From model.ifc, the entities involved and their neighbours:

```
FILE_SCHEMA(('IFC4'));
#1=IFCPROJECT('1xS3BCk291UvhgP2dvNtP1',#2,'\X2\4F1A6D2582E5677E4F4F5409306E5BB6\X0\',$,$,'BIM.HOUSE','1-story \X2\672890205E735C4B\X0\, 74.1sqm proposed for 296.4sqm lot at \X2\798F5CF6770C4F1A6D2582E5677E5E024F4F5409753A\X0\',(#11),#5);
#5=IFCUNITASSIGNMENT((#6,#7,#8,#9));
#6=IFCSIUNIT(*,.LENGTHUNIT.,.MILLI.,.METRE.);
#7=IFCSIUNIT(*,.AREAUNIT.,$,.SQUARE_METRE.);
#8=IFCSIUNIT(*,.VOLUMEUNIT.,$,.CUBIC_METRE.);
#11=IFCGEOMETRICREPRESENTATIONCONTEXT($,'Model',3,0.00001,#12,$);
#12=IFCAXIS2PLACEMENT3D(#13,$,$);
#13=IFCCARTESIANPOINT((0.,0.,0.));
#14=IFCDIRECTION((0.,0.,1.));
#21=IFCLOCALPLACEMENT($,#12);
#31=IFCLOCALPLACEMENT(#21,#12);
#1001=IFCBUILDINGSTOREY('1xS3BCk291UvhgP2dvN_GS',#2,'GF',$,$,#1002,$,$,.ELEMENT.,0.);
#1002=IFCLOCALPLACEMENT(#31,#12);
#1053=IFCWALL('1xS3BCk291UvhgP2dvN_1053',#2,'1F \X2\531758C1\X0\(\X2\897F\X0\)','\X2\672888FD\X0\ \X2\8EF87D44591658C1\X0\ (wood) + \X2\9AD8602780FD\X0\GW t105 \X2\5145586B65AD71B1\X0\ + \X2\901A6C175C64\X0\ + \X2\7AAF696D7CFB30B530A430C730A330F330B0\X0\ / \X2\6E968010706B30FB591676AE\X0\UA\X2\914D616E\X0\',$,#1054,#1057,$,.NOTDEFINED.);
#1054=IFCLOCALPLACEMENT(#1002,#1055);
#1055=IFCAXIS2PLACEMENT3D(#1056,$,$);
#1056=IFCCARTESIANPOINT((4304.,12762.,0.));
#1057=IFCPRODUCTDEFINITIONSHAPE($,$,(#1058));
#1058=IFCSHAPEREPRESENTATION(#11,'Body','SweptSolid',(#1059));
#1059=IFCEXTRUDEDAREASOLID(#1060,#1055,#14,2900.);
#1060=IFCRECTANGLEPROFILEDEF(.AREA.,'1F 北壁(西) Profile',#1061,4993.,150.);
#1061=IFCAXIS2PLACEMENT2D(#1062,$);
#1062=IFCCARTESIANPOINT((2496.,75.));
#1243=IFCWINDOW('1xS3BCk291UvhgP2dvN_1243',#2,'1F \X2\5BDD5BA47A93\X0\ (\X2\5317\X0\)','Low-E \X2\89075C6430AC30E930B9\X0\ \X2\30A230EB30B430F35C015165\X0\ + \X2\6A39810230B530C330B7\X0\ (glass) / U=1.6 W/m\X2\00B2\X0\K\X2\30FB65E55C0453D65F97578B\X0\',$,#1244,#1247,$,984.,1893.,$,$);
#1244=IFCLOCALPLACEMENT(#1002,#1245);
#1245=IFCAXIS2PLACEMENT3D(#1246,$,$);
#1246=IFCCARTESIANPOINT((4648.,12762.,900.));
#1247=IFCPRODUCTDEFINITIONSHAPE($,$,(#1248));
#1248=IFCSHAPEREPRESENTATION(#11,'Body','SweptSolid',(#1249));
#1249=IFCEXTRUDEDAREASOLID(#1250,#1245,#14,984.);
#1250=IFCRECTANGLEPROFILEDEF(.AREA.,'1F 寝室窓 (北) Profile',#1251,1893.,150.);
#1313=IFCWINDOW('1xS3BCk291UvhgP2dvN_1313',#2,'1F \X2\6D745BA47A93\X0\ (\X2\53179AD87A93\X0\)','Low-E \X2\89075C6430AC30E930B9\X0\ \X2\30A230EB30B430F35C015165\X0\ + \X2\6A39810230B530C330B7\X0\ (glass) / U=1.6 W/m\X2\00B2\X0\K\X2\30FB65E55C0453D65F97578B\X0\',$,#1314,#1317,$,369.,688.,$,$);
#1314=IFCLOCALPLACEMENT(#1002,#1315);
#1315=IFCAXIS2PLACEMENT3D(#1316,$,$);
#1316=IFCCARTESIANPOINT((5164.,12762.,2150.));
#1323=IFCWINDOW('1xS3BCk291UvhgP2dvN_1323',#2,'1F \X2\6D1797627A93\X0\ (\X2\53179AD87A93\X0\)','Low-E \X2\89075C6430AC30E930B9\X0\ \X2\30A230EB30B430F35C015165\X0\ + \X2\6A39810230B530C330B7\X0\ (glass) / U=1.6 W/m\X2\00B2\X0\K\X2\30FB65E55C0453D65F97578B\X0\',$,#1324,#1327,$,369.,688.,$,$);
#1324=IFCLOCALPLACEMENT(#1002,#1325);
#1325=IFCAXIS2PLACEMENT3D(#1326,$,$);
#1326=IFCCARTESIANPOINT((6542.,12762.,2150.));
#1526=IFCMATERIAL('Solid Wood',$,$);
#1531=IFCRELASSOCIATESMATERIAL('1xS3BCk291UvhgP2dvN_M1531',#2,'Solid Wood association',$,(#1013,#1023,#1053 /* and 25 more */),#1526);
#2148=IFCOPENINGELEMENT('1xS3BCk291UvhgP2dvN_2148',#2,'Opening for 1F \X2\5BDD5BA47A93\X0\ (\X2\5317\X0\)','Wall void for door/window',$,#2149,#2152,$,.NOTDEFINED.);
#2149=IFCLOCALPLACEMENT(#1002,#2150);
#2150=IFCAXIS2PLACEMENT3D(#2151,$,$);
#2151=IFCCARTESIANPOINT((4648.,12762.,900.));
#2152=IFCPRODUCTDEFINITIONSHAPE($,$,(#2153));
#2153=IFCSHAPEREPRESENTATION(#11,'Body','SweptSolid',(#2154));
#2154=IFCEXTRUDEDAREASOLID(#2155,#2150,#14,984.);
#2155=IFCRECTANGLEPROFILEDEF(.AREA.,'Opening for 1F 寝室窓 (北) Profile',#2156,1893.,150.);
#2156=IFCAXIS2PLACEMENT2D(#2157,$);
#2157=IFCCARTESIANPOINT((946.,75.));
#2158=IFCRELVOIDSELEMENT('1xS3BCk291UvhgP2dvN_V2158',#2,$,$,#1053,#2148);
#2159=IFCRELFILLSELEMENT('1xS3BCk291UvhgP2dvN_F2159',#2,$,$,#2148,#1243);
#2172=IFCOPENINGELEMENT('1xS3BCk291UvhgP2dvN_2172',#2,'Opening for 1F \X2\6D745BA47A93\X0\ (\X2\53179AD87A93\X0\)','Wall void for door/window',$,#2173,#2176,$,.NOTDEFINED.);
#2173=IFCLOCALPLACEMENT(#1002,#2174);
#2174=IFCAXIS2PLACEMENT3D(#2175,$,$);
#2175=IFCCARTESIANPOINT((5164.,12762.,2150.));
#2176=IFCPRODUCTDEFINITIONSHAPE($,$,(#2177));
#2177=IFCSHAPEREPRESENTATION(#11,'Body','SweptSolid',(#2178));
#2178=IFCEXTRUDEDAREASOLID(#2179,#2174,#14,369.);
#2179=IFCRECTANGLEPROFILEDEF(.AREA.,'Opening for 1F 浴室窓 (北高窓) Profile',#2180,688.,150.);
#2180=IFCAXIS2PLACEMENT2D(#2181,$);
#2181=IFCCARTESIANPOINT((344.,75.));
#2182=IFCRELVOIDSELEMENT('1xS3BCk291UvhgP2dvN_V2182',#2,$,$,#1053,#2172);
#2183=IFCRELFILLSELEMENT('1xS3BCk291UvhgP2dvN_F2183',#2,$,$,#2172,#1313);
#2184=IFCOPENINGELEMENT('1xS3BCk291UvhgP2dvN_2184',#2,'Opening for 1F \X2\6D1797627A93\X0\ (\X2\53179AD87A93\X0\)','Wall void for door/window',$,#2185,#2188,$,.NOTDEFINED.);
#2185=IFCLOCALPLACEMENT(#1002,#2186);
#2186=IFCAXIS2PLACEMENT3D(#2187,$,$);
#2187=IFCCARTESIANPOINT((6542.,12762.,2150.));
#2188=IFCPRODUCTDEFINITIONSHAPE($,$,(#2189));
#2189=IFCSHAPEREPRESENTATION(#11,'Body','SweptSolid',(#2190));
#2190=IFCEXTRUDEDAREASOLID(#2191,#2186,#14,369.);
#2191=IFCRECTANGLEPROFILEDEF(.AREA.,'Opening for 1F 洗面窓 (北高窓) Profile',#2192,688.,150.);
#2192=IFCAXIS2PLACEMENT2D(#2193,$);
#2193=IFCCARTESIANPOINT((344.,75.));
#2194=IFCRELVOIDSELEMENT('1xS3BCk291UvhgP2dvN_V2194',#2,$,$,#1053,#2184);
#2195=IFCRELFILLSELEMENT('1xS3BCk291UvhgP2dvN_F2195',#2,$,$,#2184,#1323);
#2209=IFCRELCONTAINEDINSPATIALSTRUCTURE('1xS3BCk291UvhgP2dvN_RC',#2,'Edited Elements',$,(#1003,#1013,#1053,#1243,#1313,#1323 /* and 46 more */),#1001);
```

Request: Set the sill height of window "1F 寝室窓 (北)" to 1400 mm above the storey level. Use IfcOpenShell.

```python
import numpy as np
import ifcopenshell
import ifcopenshell.api.geometry
import ifcopenshell.geom
import ifcopenshell.util.element
import ifcopenshell.util.placement
import ifcopenshell.util.shape
import ifcopenshell.util.unit

model = ifcopenshell.open("model.ifc")
unit_scale = ifcopenshell.util.unit.calculate_unit_scale(model)

window = model.by_guid("1xS3BCk291UvhgP2dvN_1243")
opening = window.FillsVoids[0].RelatingOpeningElement
storey = ifcopenshell.util.element.get_container(window, ifc_class="IfcBuildingStorey")
level = ifcopenshell.util.placement.get_local_placement(storey.ObjectPlacement)[2, 3]

# The opening's origin need not be at the sill, so measure its lowest point.
shape = ifcopenshell.geom.create_shape(ifcopenshell.geom.settings(), opening)
bottom = ifcopenshell.util.shape.get_shape_bottom_elevation(shape, shape.geometry) / unit_scale
dz = level + 1.4 / unit_scale - bottom

shift = np.array([0.0, 0.0, dz])
# The window is not placed relative to its opening, so move both.
for product in (opening, window):
    matrix = ifcopenshell.util.placement.get_local_placement(product.ObjectPlacement)
    matrix[:3, 3] += shift
    ifcopenshell.api.geometry.edit_object_placement(model, product=product, matrix=matrix, is_si=False)

print(f"moved by {dz * unit_scale:+.3f} m")

model.write("model_v2.ifc")
```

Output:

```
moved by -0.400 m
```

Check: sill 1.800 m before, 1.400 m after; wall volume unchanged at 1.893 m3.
